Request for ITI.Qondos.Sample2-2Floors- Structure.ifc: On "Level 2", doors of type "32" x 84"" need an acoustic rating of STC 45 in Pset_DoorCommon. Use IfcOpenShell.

First a look at what the model holds.

```python
import ifcopenshell
import ifcopenshell.util.element

model = ifcopenshell.open("ITI.Qondos.Sample2-2Floors- Structure.ifc")
print(model.schema)
storey = next(s for s in model.by_type("IfcBuildingStorey") if s.Name == "Level 2")
doors = [e for e in ifcopenshell.util.element.get_decomposition(storey) if e.is_a("IfcDoor")]
seen = {}
for e in doors:
    element_type = ifcopenshell.util.element.get_type(e)
    key = (element_type.Name if element_type != e and element_type else None, ifcopenshell.util.element.get_pset(e, "Pset_DoorCommon", "AcousticRating"))
    seen[key] = seen.get(key, 0) + 1
for (name, value), count in sorted(seen.items(), key=str):
    print(count, "x", name, "|", value)
```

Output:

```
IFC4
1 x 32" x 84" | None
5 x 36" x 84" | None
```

```python
import ifcopenshell
import ifcopenshell.api.pset
import ifcopenshell.util.element

model = ifcopenshell.open("ITI.Qondos.Sample2-2Floors- Structure.ifc")

storey = next(s for s in model.by_type("IfcBuildingStorey") if s.Name == "Level 2")
doors = [e for e in ifcopenshell.util.element.get_decomposition(storey) if e.is_a("IfcDoor")]

count = 0
for e in doors:
    element_type = ifcopenshell.util.element.get_type(e)
    if element_type in (None, e) or element_type.Name != '32" x 84"':
        continue
    # add_pset returns the element's existing set when there is one.
    pset = ifcopenshell.api.pset.add_pset(model, product=e, name="Pset_DoorCommon")
    ifcopenshell.api.pset.edit_pset(model, pset=pset, properties={"AcousticRating": "STC 45"})
    count += 1

print(count, "doors updated")

model.write("ITI.Qondos.Sample2-2Floors- Structure_v2.ifc")
```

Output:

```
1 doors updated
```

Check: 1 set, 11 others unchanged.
